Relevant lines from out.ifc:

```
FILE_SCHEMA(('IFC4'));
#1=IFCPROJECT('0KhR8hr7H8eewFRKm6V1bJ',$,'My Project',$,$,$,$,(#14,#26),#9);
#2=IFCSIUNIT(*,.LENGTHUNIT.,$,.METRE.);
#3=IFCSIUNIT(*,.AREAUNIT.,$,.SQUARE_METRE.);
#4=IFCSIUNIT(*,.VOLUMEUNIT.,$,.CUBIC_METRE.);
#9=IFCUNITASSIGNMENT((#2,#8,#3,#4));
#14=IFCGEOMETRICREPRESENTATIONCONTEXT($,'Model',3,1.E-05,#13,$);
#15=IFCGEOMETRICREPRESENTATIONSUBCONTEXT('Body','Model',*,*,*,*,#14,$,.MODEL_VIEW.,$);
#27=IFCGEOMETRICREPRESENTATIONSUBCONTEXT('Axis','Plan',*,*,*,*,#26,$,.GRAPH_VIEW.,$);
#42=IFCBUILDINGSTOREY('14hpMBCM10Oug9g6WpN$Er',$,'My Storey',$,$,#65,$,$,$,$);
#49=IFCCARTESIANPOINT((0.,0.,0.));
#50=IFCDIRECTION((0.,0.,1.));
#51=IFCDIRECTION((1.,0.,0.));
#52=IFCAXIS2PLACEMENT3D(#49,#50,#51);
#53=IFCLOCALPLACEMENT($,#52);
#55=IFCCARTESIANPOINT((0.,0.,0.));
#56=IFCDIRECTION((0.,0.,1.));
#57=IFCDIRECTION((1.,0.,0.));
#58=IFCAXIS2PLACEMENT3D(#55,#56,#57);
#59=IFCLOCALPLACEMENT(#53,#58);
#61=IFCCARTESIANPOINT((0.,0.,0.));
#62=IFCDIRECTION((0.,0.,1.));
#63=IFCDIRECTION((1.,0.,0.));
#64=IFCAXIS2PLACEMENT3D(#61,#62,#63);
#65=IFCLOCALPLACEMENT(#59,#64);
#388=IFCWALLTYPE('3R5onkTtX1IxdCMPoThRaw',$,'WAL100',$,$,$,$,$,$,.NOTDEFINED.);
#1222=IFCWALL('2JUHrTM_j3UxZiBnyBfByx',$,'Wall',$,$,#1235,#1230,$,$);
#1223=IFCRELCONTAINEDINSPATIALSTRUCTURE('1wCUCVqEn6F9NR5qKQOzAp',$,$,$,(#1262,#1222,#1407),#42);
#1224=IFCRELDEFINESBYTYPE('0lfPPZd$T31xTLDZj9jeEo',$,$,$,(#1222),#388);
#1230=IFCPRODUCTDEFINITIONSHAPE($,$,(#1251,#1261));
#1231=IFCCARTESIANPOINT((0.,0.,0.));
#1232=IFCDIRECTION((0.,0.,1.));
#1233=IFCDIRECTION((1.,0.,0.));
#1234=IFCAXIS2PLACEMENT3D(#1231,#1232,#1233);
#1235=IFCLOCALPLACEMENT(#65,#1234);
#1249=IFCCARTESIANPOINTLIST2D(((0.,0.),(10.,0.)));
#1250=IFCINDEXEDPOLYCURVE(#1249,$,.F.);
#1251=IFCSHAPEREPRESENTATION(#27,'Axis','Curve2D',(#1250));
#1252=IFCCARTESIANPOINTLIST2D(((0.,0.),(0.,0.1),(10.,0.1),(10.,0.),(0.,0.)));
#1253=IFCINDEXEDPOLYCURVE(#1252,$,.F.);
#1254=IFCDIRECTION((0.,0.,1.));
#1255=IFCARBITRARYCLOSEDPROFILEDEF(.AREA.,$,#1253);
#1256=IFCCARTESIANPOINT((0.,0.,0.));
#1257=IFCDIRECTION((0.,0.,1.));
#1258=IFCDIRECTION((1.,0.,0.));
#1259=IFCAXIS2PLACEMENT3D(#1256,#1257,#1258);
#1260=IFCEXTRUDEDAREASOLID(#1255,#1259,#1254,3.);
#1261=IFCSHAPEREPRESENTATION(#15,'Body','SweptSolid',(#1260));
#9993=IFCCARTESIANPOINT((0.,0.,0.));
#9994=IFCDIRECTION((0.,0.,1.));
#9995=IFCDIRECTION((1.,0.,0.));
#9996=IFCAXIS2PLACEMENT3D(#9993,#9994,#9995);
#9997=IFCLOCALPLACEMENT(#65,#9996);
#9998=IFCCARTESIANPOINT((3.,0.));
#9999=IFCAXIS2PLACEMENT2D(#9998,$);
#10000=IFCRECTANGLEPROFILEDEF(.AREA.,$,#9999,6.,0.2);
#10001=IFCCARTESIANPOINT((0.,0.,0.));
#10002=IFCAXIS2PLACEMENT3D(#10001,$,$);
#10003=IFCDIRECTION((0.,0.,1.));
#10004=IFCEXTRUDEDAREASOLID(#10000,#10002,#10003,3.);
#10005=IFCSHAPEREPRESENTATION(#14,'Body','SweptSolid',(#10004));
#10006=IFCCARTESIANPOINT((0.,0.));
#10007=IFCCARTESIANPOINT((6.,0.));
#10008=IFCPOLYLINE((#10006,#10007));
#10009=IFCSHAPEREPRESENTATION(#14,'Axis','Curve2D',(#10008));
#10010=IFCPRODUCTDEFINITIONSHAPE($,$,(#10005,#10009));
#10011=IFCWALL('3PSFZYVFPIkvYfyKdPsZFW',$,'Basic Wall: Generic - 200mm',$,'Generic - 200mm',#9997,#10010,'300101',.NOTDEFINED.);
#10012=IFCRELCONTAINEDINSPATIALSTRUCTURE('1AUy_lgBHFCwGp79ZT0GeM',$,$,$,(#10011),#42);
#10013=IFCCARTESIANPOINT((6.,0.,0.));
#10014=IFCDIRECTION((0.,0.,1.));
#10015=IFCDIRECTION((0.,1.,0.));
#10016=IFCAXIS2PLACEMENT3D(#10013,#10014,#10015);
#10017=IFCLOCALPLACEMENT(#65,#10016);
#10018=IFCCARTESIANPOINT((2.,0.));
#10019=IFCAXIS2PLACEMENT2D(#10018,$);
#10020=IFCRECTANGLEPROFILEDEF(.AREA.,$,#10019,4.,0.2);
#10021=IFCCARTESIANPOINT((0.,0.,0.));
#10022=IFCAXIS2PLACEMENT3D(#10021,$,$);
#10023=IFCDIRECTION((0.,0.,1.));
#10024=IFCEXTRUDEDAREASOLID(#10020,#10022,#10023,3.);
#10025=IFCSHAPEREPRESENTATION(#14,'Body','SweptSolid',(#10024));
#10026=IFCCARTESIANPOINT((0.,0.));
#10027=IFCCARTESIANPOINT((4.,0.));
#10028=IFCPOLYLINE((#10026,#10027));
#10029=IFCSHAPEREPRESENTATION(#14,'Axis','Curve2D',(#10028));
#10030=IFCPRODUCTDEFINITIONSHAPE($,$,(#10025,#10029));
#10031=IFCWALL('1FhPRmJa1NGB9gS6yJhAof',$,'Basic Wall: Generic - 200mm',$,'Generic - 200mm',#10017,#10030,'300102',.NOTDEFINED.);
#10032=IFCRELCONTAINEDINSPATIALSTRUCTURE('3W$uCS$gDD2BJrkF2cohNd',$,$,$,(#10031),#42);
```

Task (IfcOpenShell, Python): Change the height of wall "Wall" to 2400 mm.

```python
import ifcopenshell
import ifcopenshell.geom
import ifcopenshell.util.representation
import ifcopenshell.util.shape
import ifcopenshell.util.unit

model = ifcopenshell.open("out.ifc")
unit_scale = ifcopenshell.util.unit.calculate_unit_scale(model)
settings = ifcopenshell.geom.settings()


def volume(element):
    """Net volume in cubic metres, openings subtracted."""
    shape = ifcopenshell.geom.create_shape(settings, element)
    return ifcopenshell.util.shape.get_volume(shape.geometry)


wall = model.by_guid("2JUHrTM_j3UxZiBnyBfByx")
before = volume(wall)

body = ifcopenshell.util.representation.get_representation(wall, "Model", "Body")
solid = body.Items[0]
old_height = solid.Depth
solid.Depth = 2.4 / unit_scale
after = volume(wall)

print(f"height {old_height:g} -> {solid.Depth:g}, volume {before:.3f} -> {after:.3f} m3")

model.write("out_edited.ifc")
```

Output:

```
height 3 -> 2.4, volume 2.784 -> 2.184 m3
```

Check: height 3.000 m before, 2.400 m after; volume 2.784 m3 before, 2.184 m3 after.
